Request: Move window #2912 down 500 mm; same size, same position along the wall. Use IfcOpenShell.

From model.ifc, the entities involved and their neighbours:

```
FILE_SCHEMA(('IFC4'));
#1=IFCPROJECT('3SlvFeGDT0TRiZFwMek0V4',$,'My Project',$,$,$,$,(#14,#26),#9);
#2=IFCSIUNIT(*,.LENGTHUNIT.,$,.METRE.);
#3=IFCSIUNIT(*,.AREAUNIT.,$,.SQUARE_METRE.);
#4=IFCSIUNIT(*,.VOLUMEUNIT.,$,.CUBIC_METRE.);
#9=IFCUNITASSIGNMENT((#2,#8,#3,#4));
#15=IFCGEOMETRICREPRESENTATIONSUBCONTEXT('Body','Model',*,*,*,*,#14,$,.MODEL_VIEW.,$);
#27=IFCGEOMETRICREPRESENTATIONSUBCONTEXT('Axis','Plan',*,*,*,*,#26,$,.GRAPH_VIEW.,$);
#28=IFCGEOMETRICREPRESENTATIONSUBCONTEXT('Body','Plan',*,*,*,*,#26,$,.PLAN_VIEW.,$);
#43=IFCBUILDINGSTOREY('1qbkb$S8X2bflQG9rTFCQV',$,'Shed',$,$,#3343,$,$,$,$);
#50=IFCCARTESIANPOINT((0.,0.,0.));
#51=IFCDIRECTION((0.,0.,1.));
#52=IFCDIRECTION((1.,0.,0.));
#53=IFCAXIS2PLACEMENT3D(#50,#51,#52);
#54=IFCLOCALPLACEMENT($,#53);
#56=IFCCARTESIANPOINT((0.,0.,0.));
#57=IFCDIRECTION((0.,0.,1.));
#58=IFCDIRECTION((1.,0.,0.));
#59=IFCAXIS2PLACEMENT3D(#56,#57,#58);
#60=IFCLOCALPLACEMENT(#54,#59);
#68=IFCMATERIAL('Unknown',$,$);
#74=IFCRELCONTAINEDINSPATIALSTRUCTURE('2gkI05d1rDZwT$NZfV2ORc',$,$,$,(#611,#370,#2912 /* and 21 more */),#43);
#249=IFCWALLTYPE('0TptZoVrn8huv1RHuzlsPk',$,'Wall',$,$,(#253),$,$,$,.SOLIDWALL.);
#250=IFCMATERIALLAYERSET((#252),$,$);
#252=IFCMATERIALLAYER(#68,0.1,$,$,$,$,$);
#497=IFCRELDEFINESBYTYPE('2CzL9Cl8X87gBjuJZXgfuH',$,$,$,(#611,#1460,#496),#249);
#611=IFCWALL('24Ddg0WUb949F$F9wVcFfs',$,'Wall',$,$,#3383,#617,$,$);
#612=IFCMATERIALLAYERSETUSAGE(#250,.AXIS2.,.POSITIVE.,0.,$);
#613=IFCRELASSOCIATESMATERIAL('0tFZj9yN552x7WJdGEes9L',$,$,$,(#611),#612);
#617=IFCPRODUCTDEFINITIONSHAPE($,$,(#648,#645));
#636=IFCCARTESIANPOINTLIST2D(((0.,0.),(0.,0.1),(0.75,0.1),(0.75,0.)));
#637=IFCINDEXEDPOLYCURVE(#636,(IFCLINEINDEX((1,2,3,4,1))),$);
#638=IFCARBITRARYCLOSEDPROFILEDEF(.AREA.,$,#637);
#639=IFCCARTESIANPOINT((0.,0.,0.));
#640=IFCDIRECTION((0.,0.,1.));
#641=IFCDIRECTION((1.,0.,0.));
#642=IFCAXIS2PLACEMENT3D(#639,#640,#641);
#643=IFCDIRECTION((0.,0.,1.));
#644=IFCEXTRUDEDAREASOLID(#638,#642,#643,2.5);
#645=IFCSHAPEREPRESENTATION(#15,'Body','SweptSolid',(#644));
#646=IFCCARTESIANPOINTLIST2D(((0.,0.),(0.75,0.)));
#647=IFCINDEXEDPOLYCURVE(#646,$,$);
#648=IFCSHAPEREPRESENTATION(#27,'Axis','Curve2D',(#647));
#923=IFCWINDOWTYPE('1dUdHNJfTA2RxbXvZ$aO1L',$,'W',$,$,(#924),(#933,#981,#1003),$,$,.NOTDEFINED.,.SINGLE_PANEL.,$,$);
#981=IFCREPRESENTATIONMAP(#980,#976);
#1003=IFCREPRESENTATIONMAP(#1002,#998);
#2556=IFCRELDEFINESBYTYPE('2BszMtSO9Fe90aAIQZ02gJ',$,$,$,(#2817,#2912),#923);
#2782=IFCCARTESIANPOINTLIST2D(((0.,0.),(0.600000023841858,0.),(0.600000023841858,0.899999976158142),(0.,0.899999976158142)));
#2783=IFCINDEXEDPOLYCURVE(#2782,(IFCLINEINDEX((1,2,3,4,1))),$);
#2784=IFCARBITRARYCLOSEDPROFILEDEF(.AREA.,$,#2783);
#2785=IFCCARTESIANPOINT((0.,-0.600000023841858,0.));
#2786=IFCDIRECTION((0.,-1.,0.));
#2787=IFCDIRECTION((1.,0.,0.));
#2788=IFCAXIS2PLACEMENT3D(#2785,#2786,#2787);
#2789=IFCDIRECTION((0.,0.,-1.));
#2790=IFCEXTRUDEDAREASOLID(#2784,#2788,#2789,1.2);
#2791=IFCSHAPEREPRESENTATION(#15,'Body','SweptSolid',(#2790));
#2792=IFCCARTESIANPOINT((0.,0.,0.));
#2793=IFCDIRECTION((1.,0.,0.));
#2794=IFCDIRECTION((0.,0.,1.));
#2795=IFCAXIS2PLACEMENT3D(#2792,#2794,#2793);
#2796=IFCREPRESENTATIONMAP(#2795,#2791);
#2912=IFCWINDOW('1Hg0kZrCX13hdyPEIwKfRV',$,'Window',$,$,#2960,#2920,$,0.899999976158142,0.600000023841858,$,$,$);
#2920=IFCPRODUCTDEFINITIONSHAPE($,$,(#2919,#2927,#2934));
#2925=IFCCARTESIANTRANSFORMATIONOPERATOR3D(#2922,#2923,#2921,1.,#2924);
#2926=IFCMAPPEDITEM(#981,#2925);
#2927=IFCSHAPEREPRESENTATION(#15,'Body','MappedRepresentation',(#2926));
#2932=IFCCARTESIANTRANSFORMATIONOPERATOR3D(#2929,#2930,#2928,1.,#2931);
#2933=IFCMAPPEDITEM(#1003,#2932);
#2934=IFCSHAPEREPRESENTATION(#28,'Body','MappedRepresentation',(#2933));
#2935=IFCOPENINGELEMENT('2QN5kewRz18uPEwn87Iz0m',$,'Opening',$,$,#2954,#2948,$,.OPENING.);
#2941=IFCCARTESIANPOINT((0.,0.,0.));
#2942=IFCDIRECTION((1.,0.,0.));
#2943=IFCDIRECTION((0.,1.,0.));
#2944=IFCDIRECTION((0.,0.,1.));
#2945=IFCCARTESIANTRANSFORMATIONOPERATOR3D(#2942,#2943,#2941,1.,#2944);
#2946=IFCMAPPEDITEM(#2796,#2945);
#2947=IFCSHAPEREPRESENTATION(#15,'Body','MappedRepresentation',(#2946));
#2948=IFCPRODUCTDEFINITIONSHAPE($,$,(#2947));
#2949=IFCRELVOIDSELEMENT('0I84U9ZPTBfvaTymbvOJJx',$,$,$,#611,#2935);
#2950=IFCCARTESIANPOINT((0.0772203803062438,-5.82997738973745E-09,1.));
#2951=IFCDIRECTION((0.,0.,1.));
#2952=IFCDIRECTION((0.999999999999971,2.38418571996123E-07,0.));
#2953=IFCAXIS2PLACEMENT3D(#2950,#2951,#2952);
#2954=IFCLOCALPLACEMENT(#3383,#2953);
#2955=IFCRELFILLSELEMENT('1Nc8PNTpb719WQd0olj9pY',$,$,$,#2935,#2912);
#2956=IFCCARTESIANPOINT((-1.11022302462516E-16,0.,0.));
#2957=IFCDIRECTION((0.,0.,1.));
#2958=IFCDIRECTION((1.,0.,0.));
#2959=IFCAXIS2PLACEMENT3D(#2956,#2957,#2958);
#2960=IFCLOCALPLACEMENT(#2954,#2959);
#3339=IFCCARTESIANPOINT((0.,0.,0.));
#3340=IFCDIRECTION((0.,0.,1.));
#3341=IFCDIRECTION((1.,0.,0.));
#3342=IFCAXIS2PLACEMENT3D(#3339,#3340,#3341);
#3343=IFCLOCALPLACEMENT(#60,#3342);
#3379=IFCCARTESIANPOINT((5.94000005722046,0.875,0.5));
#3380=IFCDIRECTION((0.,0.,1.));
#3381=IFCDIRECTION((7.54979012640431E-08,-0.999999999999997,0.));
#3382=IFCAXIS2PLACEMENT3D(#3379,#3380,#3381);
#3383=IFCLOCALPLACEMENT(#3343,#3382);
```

```python
import numpy as np
import ifcopenshell
import ifcopenshell.api.geometry
import ifcopenshell.util.placement
import ifcopenshell.util.unit

model = ifcopenshell.open("model.ifc")
unit_scale = ifcopenshell.util.unit.calculate_unit_scale(model)

window = model.by_id(2912)
opening = window.FillsVoids[0].RelatingOpeningElement
dz = -0.5 / unit_scale

shift = np.array([0.0, 0.0, dz])
# The window is placed relative to its opening, so it follows when the opening moves.
matrix = ifcopenshell.util.placement.get_local_placement(opening.ObjectPlacement)
matrix[:3, 3] += shift
ifcopenshell.api.geometry.edit_object_placement(
    model, product=opening, matrix=matrix, is_si=False, should_transform_children=True
)

print(f"moved by {dz * unit_scale:+.3f} m")

model.write("model_v2.ifc")
```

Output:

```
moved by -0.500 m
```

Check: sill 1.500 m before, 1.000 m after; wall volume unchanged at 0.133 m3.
